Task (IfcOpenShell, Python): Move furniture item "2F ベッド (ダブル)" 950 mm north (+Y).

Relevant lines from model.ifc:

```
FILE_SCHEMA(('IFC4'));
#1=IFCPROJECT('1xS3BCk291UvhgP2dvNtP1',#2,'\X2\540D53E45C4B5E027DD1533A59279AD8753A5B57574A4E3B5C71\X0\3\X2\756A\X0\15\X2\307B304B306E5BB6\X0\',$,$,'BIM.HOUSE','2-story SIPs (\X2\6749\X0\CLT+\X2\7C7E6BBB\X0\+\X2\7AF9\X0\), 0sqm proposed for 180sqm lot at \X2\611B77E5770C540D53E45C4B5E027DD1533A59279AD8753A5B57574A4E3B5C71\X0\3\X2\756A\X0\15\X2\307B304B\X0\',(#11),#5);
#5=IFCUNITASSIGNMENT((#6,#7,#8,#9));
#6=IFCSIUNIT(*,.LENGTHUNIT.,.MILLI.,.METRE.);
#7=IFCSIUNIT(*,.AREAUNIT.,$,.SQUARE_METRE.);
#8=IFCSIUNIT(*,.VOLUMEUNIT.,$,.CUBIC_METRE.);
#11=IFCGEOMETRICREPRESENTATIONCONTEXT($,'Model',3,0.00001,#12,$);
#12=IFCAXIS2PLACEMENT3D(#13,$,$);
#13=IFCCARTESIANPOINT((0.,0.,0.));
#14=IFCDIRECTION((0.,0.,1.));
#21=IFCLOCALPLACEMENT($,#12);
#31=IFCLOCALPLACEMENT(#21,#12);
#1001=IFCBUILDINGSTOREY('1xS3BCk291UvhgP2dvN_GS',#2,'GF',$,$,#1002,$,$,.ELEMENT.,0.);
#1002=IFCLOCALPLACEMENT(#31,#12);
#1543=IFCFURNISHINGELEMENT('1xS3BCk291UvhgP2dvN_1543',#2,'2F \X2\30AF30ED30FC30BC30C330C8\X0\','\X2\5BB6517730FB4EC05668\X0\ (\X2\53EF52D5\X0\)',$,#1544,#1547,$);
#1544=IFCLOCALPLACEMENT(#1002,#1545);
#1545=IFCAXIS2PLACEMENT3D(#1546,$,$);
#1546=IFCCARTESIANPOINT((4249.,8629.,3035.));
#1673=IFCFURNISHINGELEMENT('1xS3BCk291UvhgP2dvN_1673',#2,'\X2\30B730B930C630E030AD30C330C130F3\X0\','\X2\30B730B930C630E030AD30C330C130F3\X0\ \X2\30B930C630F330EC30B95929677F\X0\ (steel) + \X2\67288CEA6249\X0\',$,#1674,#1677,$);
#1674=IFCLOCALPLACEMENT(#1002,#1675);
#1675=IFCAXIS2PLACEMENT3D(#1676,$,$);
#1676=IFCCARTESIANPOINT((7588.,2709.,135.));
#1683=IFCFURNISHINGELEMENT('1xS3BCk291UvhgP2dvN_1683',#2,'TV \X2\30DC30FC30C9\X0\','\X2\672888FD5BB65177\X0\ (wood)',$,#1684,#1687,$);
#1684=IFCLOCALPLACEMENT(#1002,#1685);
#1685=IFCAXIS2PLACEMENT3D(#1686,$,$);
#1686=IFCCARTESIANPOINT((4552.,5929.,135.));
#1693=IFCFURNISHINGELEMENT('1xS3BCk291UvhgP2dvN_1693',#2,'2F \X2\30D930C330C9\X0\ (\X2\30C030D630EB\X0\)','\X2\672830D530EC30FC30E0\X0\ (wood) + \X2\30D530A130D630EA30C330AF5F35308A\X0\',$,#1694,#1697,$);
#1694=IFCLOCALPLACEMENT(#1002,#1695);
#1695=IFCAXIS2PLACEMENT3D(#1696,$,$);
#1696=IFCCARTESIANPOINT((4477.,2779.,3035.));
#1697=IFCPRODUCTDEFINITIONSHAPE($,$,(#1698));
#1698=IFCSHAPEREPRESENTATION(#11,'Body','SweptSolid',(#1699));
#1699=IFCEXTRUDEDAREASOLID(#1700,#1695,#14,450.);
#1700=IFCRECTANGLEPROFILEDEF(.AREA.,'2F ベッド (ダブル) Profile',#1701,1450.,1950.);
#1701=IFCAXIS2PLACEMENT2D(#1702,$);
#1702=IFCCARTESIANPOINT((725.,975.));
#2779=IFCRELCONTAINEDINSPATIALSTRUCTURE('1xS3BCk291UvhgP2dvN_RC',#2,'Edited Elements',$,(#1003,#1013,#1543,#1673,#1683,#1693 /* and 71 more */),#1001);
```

```python
import ifcopenshell
import ifcopenshell.api.geometry
import ifcopenshell.util.placement
import ifcopenshell.util.unit

model = ifcopenshell.open("model.ifc")
unit_scale = ifcopenshell.util.unit.calculate_unit_scale(model)

item = model.by_guid("1xS3BCk291UvhgP2dvN_1693")
matrix = ifcopenshell.util.placement.get_local_placement(item.ObjectPlacement)
matrix[1, 3] += 0.95 / unit_scale
ifcopenshell.api.geometry.edit_object_placement(model, product=item, matrix=matrix, is_si=False)

print(ifcopenshell.util.placement.get_local_placement(item.ObjectPlacement).round(3) + 0.0)

model.write("model_v2.ifc")
```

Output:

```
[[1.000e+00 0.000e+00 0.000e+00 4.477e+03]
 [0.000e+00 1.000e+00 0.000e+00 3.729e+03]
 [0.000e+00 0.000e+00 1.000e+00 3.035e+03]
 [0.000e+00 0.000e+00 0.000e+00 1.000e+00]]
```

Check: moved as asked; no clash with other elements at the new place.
